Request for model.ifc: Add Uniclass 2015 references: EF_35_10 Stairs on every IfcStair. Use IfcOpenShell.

First a look at what the model holds.

```python
import ifcopenshell

model = ifcopenshell.open("model.ifc")
print(model.schema)
print("classifications:", [c.Name for c in model.by_type("IfcClassification")])
for ifc_class in ("IfcDoor", "IfcRoof", "IfcStair", "IfcWall", "IfcWindow"):
    print(ifc_class, len(model.by_type(ifc_class)))
```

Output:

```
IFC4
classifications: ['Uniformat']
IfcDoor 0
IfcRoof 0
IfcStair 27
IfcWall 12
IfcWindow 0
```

```python
import ifcopenshell
import ifcopenshell.api.classification

model = ifcopenshell.open("model.ifc")

system = ifcopenshell.api.classification.add_classification(model, classification="Uniclass 2015")

codes = {
    "IfcStair": ("EF_35_10", "Stairs"),
}
for ifc_class, (code, name) in codes.items():
    products = model.by_type(ifc_class)
    ifcopenshell.api.classification.add_reference(
        model, products=products, classification=system, identification=code, name=name
    )
    print(code, len(products))

model.write("model-out.ifc")
```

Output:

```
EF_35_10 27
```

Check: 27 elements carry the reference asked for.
